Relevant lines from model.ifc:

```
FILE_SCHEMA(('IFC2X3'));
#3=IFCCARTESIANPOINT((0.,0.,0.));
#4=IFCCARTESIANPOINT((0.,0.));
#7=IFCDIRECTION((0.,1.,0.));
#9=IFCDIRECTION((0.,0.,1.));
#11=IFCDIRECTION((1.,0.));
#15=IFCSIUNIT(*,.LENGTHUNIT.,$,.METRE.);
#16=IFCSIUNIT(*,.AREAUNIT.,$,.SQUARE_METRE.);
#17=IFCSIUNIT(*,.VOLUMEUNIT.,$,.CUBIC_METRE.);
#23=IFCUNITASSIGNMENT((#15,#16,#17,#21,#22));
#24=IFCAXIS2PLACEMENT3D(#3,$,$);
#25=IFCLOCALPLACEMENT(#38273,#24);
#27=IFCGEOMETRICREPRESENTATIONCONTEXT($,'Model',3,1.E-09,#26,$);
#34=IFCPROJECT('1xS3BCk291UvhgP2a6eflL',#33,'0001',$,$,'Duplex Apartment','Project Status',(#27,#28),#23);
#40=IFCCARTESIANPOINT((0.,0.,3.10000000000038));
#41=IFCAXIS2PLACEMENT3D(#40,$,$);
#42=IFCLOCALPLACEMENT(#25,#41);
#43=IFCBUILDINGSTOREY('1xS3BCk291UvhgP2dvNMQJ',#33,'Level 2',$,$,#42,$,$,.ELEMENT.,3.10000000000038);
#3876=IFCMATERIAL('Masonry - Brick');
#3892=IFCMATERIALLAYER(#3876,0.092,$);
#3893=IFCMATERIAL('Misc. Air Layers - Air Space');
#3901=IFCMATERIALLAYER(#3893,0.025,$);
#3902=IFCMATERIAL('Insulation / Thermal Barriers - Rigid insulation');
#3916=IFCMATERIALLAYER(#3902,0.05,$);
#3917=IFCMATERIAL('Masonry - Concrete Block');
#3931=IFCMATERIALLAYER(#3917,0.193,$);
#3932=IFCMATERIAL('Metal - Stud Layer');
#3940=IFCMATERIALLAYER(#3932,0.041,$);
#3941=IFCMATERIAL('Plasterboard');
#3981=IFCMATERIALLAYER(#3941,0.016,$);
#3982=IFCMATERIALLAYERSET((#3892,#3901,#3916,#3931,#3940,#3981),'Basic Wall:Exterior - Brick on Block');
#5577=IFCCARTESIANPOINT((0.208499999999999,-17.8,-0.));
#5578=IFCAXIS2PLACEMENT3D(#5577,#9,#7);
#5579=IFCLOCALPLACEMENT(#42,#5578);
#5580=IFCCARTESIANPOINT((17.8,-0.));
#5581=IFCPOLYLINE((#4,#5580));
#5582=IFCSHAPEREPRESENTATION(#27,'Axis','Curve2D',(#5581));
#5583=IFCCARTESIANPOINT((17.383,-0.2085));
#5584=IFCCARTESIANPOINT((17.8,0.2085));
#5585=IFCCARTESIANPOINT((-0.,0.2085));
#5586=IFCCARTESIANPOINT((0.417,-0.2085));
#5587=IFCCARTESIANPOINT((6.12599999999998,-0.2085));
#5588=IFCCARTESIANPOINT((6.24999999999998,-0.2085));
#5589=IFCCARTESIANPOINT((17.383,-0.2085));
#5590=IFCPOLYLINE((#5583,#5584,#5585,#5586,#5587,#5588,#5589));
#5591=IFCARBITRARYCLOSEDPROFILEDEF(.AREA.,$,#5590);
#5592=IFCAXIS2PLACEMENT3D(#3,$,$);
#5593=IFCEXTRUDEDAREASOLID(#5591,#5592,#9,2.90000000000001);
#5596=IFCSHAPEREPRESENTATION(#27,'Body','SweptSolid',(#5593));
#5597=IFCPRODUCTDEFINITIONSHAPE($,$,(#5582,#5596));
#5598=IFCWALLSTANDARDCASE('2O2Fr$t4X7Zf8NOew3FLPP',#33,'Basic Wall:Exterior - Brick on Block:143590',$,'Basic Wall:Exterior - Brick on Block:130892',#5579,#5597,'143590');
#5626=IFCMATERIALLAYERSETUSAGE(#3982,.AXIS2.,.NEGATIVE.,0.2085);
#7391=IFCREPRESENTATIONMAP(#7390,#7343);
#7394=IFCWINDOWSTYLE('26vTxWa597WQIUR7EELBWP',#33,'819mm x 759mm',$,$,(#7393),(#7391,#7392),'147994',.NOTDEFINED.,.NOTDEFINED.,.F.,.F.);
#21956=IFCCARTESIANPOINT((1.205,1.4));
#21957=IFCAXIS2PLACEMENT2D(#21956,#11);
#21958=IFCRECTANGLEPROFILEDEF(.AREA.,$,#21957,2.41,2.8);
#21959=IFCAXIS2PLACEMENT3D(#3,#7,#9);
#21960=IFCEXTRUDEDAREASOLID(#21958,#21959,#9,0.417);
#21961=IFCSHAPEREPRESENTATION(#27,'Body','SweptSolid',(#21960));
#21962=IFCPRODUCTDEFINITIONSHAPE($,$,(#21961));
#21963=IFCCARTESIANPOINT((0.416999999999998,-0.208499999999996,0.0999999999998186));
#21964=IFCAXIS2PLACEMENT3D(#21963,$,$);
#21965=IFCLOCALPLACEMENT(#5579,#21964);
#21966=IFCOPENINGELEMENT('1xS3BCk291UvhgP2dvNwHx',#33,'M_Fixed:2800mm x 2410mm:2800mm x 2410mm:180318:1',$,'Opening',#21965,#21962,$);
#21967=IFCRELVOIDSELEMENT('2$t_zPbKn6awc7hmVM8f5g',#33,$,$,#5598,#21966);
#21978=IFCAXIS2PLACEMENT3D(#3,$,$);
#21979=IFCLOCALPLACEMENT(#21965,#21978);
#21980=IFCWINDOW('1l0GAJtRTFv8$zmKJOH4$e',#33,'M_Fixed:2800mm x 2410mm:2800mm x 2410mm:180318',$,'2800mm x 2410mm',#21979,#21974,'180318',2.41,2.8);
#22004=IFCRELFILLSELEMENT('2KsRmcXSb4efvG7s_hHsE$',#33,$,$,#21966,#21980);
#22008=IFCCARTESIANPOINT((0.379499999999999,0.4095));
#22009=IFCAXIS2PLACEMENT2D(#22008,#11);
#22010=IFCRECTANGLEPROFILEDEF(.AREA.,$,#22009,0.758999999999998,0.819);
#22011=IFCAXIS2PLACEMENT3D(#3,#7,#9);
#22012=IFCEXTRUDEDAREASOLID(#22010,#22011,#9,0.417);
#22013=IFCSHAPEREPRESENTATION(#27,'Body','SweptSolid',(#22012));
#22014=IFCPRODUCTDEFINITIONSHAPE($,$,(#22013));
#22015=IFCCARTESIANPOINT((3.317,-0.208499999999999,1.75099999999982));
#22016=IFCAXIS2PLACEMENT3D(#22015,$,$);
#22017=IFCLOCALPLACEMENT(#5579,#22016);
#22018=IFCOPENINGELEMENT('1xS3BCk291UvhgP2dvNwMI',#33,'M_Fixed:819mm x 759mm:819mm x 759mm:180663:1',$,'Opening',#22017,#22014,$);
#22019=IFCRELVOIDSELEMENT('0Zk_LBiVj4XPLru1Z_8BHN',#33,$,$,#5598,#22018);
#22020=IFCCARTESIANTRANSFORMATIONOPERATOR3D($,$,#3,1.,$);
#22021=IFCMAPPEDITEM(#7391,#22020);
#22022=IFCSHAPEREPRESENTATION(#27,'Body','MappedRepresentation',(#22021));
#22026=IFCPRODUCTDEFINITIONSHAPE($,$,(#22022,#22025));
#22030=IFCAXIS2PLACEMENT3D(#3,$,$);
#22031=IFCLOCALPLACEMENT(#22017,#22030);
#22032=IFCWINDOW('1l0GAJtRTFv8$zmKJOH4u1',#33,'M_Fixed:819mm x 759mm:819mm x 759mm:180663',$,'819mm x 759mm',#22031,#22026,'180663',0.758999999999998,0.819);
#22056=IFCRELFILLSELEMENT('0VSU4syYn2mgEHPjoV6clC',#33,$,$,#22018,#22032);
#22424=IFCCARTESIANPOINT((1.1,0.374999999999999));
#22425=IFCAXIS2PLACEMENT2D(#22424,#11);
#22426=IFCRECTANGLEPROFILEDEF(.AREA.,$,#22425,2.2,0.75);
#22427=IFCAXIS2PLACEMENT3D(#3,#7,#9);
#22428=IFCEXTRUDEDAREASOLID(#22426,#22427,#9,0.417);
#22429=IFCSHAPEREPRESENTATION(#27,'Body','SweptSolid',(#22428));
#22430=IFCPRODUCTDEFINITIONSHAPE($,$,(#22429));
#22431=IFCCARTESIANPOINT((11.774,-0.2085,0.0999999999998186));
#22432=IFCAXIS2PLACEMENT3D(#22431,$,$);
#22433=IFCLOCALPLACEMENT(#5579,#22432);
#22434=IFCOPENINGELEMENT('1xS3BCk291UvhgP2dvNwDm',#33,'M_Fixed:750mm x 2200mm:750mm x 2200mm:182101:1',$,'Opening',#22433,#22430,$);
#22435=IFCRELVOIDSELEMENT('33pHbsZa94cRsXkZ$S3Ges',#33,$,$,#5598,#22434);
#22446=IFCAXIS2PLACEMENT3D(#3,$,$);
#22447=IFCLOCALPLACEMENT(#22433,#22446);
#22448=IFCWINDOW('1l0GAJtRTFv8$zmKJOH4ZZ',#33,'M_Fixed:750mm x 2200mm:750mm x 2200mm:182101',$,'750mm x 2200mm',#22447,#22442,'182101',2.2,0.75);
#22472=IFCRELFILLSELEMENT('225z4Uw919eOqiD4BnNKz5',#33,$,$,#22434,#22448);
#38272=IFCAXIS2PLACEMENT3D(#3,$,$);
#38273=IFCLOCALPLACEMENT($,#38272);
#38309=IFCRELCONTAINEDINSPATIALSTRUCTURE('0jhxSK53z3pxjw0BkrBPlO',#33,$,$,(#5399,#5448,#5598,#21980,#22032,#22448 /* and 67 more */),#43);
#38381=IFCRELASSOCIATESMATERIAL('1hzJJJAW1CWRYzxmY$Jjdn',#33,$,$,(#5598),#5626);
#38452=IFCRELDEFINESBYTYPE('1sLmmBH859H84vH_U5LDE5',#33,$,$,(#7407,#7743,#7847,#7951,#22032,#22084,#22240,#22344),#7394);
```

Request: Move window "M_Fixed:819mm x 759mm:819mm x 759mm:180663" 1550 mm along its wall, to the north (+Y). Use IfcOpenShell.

```python
import ifcopenshell
import ifcopenshell.api.geometry
import ifcopenshell.util.placement
import ifcopenshell.util.unit

model = ifcopenshell.open("model.ifc")
unit_scale = ifcopenshell.util.unit.calculate_unit_scale(model)

window = model.by_id(22032)
opening = window.FillsVoids[0].RelatingOpeningElement
wall = opening.VoidsElements[0].RelatingBuildingElement

wall_matrix = ifcopenshell.util.placement.get_local_placement(wall.ObjectPlacement)
shift = wall_matrix[:3, 0] * 1.55 / unit_scale
before = ifcopenshell.util.placement.get_local_placement(window.ObjectPlacement)[:3, 3].copy()

# The window is placed relative to its opening, so it follows when the opening moves.
matrix = ifcopenshell.util.placement.get_local_placement(opening.ObjectPlacement)
matrix[:3, 3] += shift
ifcopenshell.api.geometry.edit_object_placement(
    model, product=opening, matrix=matrix, is_si=False, should_transform_children=True
)

after = ifcopenshell.util.placement.get_local_placement(window.ObjectPlacement)[:3, 3]
print("window moved by", (after - before).round(3) + 0.0)

model.write("model-out.ifc")
```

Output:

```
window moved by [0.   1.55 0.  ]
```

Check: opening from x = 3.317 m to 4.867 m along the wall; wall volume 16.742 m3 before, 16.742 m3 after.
